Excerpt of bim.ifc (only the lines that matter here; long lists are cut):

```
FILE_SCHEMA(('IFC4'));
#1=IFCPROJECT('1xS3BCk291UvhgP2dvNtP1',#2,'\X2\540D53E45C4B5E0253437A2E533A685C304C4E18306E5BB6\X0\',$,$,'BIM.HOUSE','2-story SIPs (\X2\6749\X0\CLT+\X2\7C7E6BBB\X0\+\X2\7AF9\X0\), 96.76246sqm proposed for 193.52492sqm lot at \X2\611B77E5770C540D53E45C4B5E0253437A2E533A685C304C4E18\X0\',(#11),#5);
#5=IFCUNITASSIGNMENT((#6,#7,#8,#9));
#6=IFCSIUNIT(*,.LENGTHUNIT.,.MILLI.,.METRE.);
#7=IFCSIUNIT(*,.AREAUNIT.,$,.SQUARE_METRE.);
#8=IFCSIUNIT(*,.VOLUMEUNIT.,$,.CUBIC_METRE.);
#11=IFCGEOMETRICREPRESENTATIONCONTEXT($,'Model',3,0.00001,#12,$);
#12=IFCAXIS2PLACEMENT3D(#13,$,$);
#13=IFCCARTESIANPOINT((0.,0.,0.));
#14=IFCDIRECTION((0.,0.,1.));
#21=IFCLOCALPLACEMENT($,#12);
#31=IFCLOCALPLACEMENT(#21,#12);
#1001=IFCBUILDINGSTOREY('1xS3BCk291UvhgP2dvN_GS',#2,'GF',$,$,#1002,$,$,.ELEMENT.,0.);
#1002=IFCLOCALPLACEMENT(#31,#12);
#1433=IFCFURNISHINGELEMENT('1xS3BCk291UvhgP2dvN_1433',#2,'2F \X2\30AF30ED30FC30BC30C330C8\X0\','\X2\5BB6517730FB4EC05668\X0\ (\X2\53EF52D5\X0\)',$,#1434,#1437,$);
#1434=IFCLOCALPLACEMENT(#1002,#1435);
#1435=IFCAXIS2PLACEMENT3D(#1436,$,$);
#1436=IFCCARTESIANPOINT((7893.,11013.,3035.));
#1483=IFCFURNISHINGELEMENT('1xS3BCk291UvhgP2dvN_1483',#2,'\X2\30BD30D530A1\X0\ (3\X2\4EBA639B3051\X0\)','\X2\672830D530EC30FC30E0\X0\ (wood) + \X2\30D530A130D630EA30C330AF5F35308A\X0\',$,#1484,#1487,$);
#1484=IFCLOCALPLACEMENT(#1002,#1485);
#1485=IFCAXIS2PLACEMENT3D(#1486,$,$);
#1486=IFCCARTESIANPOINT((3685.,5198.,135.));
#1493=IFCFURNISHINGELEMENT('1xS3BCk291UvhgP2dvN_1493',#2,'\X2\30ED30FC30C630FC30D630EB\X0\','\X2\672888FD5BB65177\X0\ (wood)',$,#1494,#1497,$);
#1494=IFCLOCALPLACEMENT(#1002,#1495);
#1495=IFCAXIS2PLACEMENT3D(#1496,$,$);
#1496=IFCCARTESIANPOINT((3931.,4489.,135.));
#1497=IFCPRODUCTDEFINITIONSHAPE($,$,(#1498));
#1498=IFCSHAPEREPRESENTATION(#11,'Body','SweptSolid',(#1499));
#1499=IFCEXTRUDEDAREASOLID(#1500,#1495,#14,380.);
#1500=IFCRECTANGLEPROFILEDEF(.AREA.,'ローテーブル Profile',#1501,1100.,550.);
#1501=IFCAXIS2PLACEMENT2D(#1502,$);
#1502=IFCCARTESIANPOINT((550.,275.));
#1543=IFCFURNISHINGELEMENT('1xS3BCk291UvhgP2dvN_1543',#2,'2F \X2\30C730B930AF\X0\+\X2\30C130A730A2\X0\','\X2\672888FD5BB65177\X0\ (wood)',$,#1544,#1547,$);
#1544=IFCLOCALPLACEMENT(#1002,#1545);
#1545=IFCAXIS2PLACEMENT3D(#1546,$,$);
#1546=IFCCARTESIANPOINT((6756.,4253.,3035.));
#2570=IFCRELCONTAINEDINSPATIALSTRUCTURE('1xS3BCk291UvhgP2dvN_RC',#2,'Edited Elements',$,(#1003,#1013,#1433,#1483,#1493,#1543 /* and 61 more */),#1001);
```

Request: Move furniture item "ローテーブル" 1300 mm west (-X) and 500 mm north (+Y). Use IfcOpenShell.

```python
import ifcopenshell
import ifcopenshell.api.geometry
import ifcopenshell.util.placement
import ifcopenshell.util.unit

model = ifcopenshell.open("bim.ifc")
unit_scale = ifcopenshell.util.unit.calculate_unit_scale(model)

item = model.by_id(1493)
matrix = ifcopenshell.util.placement.get_local_placement(item.ObjectPlacement)
matrix[0, 3] -= 1.3 / unit_scale
matrix[1, 3] += 0.5 / unit_scale
ifcopenshell.api.geometry.edit_object_placement(model, product=item, matrix=matrix, is_si=False)

print(ifcopenshell.util.placement.get_local_placement(item.ObjectPlacement).round(3) + 0.0)

model.write("bim_updated.ifc")
```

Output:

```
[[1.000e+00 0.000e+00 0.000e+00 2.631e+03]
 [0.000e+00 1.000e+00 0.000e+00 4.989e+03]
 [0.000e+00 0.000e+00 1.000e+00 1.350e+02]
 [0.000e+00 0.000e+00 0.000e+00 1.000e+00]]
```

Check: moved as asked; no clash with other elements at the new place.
